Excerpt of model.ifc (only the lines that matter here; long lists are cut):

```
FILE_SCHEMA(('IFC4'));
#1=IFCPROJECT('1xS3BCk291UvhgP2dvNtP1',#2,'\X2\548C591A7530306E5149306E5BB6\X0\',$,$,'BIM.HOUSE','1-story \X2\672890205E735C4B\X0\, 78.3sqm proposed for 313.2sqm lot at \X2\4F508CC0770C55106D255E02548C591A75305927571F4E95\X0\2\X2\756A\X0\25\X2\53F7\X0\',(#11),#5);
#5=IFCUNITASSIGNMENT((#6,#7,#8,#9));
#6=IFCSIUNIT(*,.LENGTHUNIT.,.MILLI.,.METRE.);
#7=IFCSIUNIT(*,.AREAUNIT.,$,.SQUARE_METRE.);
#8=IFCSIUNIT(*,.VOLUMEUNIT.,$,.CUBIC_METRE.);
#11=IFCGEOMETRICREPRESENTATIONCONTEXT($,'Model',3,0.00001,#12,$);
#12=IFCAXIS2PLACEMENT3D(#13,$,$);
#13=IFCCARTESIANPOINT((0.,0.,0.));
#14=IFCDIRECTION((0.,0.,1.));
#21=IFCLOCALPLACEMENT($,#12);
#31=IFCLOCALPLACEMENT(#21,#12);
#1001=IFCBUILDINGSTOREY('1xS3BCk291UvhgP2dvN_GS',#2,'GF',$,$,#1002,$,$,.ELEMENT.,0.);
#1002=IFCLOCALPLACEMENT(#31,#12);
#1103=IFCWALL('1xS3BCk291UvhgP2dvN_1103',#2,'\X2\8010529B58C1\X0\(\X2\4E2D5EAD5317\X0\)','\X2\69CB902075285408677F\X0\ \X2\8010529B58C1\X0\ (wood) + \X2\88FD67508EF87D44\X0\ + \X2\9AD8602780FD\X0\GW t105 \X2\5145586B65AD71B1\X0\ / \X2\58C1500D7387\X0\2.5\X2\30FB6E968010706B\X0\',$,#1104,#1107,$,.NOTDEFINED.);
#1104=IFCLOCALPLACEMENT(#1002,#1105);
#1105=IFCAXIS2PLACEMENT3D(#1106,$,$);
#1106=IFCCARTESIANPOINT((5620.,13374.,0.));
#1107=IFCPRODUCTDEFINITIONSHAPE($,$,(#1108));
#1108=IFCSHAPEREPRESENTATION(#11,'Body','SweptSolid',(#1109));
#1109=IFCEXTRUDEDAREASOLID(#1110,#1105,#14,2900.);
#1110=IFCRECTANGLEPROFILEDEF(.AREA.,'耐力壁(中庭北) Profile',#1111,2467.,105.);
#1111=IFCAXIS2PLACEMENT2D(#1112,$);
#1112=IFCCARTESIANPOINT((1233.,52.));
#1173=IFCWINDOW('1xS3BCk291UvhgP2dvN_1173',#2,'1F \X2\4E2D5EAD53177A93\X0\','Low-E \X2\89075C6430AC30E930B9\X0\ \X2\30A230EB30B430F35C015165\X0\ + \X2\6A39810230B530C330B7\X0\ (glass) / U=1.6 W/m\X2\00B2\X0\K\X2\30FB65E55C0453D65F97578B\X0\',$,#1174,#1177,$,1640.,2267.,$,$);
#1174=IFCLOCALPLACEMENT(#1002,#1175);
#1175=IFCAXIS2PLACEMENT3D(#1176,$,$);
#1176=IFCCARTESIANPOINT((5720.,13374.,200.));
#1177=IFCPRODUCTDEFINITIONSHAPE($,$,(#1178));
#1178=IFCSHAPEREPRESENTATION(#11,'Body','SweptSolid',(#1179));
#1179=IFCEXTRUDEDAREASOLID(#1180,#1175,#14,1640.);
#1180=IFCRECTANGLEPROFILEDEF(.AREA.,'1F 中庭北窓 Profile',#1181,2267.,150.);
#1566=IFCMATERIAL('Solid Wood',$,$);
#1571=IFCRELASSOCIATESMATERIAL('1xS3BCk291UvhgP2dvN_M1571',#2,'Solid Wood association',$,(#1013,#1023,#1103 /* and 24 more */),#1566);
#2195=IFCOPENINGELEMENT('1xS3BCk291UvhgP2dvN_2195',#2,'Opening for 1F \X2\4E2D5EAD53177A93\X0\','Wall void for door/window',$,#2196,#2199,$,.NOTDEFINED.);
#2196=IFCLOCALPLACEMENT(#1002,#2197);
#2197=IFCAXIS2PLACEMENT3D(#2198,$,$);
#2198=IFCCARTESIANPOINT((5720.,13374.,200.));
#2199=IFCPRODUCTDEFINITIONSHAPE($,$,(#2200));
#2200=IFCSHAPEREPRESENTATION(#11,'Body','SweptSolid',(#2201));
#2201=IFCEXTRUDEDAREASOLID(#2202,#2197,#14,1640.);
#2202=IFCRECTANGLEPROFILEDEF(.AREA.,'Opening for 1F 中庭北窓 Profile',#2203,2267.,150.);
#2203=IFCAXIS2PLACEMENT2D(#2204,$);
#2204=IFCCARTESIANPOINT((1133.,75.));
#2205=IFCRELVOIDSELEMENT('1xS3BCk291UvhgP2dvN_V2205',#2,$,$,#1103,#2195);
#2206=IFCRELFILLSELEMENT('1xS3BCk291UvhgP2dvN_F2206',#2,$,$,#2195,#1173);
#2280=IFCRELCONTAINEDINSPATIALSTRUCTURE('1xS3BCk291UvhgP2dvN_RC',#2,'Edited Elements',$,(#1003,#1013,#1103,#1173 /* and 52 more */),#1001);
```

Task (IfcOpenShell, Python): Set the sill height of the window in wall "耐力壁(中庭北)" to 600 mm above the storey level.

```python
import numpy as np
import ifcopenshell
import ifcopenshell.api.geometry
import ifcopenshell.geom
import ifcopenshell.util.element
import ifcopenshell.util.placement
import ifcopenshell.util.shape
import ifcopenshell.util.unit

model = ifcopenshell.open("model.ifc")
unit_scale = ifcopenshell.util.unit.calculate_unit_scale(model)

window = model.by_id(1173)
opening = window.FillsVoids[0].RelatingOpeningElement
storey = ifcopenshell.util.element.get_container(window, ifc_class="IfcBuildingStorey")
level = ifcopenshell.util.placement.get_local_placement(storey.ObjectPlacement)[2, 3]

# The opening's origin need not be at the sill, so measure its lowest point.
shape = ifcopenshell.geom.create_shape(ifcopenshell.geom.settings(), opening)
bottom = ifcopenshell.util.shape.get_shape_bottom_elevation(shape, shape.geometry) / unit_scale
dz = level + 0.6 / unit_scale - bottom

shift = np.array([0.0, 0.0, dz])
# The window is not placed relative to its opening, so move both.
for product in (opening, window):
    matrix = ifcopenshell.util.placement.get_local_placement(product.ObjectPlacement)
    matrix[:3, 3] += shift
    ifcopenshell.api.geometry.edit_object_placement(model, product=product, matrix=matrix, is_si=False)

print(f"moved by {dz * unit_scale:+.3f} m")

model.write("model_v2.ifc")
```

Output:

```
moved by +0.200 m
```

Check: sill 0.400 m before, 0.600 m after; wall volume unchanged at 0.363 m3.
